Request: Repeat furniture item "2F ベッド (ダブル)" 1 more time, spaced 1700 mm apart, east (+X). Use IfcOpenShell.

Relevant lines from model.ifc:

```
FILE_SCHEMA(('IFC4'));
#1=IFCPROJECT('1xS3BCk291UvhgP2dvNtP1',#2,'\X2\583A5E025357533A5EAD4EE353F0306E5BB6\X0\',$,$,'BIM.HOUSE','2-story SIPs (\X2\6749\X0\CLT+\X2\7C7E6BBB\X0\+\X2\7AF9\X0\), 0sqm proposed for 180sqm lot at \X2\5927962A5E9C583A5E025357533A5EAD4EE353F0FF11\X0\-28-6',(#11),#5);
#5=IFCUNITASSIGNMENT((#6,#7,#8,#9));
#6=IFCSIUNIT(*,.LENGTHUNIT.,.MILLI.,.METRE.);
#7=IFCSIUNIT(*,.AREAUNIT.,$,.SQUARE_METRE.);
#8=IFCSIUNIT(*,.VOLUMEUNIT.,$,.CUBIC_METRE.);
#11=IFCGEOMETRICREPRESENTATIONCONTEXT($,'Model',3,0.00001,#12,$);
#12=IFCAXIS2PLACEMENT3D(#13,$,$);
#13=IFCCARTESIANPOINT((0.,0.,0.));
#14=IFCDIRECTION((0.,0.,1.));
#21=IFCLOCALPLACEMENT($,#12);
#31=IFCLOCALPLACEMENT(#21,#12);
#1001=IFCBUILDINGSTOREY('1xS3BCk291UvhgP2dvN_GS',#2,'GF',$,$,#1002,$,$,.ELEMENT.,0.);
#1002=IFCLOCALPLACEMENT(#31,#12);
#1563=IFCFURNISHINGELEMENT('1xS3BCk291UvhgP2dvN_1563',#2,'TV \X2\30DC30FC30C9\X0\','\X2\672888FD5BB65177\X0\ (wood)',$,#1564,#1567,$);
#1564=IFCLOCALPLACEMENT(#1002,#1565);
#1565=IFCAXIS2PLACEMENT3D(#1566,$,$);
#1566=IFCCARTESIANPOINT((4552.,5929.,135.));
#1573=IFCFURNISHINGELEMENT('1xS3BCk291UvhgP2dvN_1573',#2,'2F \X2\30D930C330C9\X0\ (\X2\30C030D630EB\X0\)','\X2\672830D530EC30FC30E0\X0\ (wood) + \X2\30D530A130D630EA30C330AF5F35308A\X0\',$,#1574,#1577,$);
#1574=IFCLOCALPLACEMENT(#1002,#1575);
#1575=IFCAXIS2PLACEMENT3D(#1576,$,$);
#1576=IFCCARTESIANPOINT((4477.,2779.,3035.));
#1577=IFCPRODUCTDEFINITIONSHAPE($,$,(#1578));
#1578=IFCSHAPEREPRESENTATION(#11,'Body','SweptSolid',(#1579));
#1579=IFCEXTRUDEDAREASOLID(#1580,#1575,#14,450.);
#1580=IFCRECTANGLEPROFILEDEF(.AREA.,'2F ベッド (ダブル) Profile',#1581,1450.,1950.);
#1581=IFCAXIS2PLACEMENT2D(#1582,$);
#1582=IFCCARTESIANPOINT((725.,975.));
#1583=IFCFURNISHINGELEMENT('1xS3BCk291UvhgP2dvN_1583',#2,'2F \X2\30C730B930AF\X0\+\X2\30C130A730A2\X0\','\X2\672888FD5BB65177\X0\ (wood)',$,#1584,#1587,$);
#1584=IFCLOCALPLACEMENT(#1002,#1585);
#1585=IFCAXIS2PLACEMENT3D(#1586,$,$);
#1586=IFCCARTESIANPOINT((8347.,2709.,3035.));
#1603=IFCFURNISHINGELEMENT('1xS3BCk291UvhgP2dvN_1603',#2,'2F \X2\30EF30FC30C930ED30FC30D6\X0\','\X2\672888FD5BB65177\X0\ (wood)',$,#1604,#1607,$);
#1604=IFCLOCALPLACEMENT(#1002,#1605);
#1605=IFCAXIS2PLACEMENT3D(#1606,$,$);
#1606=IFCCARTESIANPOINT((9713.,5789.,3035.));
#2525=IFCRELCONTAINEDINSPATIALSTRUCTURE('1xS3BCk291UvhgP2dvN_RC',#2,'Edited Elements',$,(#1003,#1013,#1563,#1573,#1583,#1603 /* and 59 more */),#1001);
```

```python
import numpy as np
import ifcopenshell
import ifcopenshell.api.geometry
import ifcopenshell.api.root
import ifcopenshell.util.element
import ifcopenshell.util.placement
import ifcopenshell.util.unit

model = ifcopenshell.open("model.ifc")
unit_scale = ifcopenshell.util.unit.calculate_unit_scale(model)


def reuse_history(source, copy):
    """copy_class also copies each property set's owner history, people and application; keep the originals."""
    for rel in copy.IsDefinedBy:
        if rel.is_a("IfcRelDefinesByProperties") and (history := rel.RelatingPropertyDefinition.OwnerHistory):
            rel.RelatingPropertyDefinition.OwnerHistory = source.OwnerHistory
            ifcopenshell.util.element.remove_deep2(model, history)


source = model.by_guid("1xS3BCk291UvhgP2dvN_1573")
base = ifcopenshell.util.placement.get_local_placement(source.ObjectPlacement)
step = np.array([1.0, 0.0, 0.0]) * 1.7 / unit_scale

for i in range(1, 2):
    copy = ifcopenshell.api.root.copy_class(model, product=source)
    copy.Representation = ifcopenshell.util.element.copy_deep(
        model, source.Representation, exclude=["IfcGeometricRepresentationContext", "IfcRepresentationMap"]
    )
    reuse_history(source, copy)
    matrix = base.copy()
    matrix[:3, 3] += i * step
    print("added at", matrix[:3, 3].round(3) + 0.0)
    ifcopenshell.api.geometry.edit_object_placement(model, product=copy, matrix=matrix, is_si=False)

model.write("model_rev.ifc")
```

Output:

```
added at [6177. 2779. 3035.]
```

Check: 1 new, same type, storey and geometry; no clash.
